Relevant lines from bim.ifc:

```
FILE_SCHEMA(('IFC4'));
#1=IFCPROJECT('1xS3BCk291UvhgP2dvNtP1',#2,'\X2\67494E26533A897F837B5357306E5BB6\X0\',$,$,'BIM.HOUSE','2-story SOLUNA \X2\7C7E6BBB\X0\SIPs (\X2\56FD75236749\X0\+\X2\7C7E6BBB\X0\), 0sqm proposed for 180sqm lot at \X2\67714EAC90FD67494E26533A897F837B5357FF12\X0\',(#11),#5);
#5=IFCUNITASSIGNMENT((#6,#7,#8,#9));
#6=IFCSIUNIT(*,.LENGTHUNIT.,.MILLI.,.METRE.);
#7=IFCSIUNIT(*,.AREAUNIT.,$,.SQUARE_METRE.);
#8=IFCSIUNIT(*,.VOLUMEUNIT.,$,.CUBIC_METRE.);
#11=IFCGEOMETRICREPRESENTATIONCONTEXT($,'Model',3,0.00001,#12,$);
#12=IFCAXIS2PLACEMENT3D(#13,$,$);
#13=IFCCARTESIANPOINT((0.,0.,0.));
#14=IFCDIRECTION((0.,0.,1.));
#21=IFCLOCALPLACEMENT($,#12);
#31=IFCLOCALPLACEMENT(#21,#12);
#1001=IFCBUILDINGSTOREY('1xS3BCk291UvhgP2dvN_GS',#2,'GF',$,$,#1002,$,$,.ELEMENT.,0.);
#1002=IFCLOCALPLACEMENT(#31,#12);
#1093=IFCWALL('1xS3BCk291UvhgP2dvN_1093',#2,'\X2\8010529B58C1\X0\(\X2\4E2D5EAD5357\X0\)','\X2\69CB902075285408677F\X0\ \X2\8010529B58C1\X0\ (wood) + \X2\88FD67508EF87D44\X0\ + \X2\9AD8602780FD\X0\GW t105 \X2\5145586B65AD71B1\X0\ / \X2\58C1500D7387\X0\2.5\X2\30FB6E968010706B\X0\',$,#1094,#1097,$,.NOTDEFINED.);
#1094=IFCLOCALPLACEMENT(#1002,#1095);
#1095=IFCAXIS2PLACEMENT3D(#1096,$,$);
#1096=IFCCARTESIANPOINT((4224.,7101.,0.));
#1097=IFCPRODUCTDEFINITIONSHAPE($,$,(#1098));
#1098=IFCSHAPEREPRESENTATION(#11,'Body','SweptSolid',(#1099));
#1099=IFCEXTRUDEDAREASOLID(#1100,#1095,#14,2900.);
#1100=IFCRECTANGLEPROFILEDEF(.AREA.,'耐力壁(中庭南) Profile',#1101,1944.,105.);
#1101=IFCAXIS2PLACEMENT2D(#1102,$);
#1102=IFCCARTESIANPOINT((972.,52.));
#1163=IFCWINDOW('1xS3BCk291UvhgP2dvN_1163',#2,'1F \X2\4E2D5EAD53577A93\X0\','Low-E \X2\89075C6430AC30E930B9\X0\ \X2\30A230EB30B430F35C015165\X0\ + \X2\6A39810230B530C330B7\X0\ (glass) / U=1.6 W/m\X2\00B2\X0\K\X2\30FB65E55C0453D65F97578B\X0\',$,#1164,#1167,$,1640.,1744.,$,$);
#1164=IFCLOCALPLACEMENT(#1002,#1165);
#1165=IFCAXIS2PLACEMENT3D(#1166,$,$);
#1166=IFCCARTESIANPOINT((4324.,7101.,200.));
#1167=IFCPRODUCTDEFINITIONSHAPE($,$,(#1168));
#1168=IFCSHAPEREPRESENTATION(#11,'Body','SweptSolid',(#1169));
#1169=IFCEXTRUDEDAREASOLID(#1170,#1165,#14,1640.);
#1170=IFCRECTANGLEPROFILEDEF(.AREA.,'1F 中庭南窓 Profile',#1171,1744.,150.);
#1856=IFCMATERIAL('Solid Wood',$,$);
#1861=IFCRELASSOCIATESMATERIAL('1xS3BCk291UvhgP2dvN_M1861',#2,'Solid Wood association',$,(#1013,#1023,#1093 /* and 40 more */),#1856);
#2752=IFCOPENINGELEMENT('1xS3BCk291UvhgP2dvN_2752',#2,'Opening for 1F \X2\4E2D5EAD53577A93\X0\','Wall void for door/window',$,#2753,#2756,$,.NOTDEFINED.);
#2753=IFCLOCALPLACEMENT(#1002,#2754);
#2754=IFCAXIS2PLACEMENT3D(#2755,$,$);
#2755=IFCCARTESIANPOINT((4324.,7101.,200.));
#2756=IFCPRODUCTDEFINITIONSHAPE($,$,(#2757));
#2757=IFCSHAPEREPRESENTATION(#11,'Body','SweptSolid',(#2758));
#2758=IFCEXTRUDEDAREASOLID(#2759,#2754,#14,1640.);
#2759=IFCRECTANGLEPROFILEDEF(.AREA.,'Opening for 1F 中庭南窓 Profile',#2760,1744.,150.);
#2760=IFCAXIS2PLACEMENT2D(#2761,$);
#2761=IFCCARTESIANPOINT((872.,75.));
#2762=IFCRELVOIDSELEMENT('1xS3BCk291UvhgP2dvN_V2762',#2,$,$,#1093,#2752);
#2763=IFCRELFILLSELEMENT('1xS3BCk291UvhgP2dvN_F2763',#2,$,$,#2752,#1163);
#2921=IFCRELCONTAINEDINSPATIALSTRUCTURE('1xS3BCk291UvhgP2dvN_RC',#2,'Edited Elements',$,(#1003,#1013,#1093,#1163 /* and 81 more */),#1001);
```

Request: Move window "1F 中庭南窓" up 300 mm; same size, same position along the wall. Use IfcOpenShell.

```python
import numpy as np
import ifcopenshell
import ifcopenshell.api.geometry
import ifcopenshell.util.placement
import ifcopenshell.util.unit

model = ifcopenshell.open("bim.ifc")
unit_scale = ifcopenshell.util.unit.calculate_unit_scale(model)

window = model.by_guid("1xS3BCk291UvhgP2dvN_1163")
opening = window.FillsVoids[0].RelatingOpeningElement
dz = 0.3 / unit_scale

shift = np.array([0.0, 0.0, dz])
# The window is not placed relative to its opening, so move both.
for product in (opening, window):
    matrix = ifcopenshell.util.placement.get_local_placement(product.ObjectPlacement)
    matrix[:3, 3] += shift
    ifcopenshell.api.geometry.edit_object_placement(model, product=product, matrix=matrix, is_si=False)

print(f"moved by {dz * unit_scale:+.3f} m")

model.write("bim_rev.ifc")
```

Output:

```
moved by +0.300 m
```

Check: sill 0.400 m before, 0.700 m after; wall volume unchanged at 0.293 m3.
